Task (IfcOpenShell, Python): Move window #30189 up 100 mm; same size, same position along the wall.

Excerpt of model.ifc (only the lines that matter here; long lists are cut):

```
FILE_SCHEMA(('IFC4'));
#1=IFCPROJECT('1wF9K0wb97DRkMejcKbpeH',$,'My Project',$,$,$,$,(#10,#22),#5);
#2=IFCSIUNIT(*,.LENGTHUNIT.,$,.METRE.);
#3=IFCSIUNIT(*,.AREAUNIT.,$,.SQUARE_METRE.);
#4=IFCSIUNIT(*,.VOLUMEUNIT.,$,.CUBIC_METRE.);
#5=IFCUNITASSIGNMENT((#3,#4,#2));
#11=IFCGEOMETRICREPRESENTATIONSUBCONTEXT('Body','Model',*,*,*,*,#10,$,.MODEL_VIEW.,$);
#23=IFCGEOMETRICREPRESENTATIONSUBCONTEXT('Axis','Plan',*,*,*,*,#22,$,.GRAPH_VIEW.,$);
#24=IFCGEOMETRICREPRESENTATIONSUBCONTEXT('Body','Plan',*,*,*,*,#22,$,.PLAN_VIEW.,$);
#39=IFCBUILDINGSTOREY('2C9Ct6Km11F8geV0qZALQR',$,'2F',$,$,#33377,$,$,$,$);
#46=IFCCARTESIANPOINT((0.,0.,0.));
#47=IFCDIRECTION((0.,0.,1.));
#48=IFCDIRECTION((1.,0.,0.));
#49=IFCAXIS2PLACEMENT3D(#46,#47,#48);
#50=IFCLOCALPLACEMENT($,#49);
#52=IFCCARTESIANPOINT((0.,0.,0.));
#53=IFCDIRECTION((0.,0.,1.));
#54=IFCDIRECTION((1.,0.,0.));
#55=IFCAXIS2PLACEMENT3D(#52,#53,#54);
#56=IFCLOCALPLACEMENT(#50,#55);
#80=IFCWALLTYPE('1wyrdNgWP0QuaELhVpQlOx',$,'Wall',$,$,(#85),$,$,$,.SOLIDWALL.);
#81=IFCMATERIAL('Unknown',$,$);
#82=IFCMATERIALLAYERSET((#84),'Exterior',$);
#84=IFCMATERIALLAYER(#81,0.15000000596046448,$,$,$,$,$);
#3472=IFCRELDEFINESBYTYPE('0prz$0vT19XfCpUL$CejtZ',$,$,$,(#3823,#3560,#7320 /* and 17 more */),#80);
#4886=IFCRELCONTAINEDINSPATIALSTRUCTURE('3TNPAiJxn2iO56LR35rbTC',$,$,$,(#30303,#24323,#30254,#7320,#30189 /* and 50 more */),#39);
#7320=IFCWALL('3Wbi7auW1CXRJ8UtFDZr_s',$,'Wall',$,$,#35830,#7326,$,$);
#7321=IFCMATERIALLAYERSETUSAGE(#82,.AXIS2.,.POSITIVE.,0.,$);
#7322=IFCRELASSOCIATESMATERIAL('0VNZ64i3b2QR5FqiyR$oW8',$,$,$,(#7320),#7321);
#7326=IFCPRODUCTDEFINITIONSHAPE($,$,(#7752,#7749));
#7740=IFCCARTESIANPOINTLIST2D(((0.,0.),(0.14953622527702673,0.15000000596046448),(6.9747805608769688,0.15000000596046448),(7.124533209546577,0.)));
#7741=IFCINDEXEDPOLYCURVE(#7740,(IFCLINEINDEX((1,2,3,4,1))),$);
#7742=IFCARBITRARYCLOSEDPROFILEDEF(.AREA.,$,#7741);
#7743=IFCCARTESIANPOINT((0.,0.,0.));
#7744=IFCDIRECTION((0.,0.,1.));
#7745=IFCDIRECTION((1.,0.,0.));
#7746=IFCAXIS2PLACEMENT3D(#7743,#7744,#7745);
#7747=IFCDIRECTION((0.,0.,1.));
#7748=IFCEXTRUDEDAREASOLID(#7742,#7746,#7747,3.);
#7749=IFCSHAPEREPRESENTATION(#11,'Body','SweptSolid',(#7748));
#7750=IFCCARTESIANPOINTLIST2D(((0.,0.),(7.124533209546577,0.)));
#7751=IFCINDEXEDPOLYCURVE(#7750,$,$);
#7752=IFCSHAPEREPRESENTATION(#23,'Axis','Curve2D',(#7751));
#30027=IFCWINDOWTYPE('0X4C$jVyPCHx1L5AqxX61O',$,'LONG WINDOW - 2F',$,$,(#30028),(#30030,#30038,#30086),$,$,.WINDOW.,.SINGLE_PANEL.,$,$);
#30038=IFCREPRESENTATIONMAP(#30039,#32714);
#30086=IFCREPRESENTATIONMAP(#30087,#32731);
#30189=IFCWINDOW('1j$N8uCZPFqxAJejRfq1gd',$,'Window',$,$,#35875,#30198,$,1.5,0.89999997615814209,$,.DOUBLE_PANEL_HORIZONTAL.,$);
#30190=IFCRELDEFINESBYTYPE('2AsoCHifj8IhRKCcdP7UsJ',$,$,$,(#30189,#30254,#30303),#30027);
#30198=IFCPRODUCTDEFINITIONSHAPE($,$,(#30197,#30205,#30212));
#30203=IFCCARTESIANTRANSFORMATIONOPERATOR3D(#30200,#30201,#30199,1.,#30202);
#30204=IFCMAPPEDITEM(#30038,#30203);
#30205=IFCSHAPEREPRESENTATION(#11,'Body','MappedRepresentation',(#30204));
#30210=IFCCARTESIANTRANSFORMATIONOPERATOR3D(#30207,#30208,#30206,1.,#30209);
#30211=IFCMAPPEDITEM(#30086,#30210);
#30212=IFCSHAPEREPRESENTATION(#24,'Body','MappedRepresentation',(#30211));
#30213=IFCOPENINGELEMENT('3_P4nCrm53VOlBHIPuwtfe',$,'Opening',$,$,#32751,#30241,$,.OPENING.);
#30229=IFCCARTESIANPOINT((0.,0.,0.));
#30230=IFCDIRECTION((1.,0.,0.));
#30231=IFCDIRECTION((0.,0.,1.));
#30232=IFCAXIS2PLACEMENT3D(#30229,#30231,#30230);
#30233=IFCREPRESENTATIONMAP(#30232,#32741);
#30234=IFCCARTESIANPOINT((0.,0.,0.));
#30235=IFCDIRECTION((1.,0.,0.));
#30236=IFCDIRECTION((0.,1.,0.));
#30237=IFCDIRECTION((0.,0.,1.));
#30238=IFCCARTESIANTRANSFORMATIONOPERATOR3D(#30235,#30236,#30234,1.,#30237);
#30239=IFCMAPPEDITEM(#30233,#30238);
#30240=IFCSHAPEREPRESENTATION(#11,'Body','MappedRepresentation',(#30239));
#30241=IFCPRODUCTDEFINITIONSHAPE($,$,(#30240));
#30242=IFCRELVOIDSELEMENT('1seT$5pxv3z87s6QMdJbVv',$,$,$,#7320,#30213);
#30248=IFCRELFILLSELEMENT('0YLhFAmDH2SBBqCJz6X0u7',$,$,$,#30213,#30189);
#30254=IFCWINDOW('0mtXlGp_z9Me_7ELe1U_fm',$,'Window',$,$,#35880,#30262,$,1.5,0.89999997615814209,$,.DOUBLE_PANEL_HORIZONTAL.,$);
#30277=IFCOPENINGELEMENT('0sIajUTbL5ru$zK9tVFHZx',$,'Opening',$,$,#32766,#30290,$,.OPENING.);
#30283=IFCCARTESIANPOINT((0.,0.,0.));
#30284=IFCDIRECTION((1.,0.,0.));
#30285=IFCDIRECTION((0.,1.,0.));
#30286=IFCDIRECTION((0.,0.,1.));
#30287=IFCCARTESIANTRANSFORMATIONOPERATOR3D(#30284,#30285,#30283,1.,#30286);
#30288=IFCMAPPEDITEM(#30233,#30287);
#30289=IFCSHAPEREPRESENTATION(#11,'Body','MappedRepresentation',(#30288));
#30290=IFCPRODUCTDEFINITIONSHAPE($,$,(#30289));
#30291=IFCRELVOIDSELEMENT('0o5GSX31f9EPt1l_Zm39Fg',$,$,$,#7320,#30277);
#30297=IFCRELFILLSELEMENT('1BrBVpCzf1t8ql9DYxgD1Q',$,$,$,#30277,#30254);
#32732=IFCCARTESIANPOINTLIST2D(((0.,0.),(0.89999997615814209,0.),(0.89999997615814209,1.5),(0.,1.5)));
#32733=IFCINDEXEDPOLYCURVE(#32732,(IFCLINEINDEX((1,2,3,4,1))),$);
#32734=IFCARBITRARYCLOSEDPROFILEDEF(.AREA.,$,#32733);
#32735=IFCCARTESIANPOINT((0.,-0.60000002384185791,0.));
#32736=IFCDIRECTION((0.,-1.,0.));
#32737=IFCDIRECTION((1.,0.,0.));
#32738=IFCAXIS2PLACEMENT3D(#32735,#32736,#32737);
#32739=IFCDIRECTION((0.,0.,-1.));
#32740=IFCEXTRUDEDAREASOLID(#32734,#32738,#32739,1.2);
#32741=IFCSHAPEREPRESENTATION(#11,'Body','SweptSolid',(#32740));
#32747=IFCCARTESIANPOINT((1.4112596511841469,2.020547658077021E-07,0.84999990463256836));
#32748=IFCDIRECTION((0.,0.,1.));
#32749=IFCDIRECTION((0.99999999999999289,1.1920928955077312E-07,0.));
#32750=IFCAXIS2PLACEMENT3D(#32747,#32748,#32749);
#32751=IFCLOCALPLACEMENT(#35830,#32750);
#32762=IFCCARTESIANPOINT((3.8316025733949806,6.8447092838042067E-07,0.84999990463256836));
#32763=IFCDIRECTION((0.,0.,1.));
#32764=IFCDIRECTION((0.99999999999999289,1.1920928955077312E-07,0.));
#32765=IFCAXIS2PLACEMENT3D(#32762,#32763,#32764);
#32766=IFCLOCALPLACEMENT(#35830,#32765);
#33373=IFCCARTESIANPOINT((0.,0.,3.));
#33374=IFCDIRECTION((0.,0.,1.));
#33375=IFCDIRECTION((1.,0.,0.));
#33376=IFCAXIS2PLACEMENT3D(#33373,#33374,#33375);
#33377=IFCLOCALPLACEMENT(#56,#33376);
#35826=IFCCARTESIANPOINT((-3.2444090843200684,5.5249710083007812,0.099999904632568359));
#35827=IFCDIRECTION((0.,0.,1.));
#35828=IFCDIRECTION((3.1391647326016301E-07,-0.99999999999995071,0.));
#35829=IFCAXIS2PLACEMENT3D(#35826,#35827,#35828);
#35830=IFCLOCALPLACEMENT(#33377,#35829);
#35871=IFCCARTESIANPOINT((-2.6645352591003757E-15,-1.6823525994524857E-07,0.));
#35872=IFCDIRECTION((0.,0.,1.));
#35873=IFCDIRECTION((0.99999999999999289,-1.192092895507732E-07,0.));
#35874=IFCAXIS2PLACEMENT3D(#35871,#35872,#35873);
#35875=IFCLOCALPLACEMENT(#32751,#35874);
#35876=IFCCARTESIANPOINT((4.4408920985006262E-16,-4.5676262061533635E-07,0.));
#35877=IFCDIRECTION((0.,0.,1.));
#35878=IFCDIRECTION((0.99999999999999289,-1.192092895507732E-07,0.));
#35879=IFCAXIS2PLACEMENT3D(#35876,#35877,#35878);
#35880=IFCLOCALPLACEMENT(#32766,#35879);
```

```python
import numpy as np
import ifcopenshell
import ifcopenshell.api.geometry
import ifcopenshell.util.placement
import ifcopenshell.util.unit

model = ifcopenshell.open("model.ifc")
unit_scale = ifcopenshell.util.unit.calculate_unit_scale(model)

window = model.by_guid("1j$N8uCZPFqxAJejRfq1gd")
opening = window.FillsVoids[0].RelatingOpeningElement
dz = 0.1

shift = np.array([0.0, 0.0, dz])
# The window is placed relative to its opening, so it follows when the opening moves.
matrix = ifcopenshell.util.placement.get_local_placement(opening.ObjectPlacement)
matrix[:3, 3] += shift
ifcopenshell.api.geometry.edit_object_placement(
    model, product=opening, matrix=matrix, is_si=False, should_transform_children=True
)

print(f"moved by {dz * unit_scale:+.3f} m")

model.write("model_v2.ifc")
```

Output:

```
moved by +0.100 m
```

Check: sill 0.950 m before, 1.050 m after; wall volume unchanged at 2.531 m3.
